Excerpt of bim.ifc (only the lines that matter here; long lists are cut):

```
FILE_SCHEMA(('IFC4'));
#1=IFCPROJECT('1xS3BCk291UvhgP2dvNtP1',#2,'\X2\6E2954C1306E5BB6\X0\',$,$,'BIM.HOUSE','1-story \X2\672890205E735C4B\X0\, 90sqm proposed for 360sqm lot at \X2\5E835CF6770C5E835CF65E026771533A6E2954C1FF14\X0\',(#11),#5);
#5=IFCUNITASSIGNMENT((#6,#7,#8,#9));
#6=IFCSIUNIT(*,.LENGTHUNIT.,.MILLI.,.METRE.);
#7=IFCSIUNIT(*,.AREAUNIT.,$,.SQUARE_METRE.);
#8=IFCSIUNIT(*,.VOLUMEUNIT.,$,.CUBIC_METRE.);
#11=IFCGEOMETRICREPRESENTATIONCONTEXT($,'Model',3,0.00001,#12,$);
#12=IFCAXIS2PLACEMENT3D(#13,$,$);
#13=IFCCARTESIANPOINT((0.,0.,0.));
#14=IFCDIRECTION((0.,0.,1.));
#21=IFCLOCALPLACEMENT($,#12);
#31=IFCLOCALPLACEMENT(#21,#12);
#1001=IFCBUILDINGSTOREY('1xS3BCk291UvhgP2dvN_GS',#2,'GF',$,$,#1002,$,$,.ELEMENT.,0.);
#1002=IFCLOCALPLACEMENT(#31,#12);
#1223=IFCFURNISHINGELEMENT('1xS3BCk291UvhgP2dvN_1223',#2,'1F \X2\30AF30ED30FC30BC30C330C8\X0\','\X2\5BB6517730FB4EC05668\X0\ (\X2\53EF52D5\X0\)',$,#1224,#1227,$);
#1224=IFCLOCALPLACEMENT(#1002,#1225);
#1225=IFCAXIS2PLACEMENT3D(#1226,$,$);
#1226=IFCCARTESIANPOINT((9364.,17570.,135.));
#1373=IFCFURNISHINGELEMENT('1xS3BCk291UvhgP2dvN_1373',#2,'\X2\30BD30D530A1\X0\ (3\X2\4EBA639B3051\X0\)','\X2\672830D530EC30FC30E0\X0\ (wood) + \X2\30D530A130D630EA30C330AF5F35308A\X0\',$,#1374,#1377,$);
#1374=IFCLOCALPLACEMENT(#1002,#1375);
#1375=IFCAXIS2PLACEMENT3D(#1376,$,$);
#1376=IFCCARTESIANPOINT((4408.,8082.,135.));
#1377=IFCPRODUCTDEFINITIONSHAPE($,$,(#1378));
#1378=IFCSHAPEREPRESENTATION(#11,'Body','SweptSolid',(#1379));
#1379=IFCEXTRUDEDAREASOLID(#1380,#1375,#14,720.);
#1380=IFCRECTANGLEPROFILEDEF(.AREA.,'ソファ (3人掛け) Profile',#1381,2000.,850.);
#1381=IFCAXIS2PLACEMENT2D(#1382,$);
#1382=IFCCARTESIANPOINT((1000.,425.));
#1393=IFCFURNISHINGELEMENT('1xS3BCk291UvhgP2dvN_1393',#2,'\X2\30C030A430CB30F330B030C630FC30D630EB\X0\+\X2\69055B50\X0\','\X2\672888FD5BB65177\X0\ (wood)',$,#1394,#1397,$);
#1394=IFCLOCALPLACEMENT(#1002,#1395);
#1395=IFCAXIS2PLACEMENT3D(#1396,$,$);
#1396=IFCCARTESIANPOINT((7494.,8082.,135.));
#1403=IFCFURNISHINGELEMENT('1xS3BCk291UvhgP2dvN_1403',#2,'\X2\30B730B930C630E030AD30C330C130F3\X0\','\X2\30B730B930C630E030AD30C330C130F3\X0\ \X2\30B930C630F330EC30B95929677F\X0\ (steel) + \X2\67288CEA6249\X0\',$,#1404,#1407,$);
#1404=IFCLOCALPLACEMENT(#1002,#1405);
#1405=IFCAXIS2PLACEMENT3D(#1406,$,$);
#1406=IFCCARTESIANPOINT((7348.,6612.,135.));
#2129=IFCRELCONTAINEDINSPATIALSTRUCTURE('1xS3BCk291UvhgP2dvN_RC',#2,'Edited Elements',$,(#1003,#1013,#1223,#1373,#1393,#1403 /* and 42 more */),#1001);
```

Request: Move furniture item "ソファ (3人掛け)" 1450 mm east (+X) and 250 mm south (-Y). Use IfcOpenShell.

```python
import ifcopenshell
import ifcopenshell.api.geometry
import ifcopenshell.util.placement

model = ifcopenshell.open("bim.ifc")

item = model.by_guid("1xS3BCk291UvhgP2dvN_1373")
matrix = ifcopenshell.util.placement.get_local_placement(item.ObjectPlacement)
matrix[0, 3] += 1450.0
matrix[1, 3] -= 250.0
ifcopenshell.api.geometry.edit_object_placement(model, product=item, matrix=matrix, is_si=False)

print(ifcopenshell.util.placement.get_local_placement(item.ObjectPlacement).round(3) + 0.0)

model.write("bim_v2.ifc")
```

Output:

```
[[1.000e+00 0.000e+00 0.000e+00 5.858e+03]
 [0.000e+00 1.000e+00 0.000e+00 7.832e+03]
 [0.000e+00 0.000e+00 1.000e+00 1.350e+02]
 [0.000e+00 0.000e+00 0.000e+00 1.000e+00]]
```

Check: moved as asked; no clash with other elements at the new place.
